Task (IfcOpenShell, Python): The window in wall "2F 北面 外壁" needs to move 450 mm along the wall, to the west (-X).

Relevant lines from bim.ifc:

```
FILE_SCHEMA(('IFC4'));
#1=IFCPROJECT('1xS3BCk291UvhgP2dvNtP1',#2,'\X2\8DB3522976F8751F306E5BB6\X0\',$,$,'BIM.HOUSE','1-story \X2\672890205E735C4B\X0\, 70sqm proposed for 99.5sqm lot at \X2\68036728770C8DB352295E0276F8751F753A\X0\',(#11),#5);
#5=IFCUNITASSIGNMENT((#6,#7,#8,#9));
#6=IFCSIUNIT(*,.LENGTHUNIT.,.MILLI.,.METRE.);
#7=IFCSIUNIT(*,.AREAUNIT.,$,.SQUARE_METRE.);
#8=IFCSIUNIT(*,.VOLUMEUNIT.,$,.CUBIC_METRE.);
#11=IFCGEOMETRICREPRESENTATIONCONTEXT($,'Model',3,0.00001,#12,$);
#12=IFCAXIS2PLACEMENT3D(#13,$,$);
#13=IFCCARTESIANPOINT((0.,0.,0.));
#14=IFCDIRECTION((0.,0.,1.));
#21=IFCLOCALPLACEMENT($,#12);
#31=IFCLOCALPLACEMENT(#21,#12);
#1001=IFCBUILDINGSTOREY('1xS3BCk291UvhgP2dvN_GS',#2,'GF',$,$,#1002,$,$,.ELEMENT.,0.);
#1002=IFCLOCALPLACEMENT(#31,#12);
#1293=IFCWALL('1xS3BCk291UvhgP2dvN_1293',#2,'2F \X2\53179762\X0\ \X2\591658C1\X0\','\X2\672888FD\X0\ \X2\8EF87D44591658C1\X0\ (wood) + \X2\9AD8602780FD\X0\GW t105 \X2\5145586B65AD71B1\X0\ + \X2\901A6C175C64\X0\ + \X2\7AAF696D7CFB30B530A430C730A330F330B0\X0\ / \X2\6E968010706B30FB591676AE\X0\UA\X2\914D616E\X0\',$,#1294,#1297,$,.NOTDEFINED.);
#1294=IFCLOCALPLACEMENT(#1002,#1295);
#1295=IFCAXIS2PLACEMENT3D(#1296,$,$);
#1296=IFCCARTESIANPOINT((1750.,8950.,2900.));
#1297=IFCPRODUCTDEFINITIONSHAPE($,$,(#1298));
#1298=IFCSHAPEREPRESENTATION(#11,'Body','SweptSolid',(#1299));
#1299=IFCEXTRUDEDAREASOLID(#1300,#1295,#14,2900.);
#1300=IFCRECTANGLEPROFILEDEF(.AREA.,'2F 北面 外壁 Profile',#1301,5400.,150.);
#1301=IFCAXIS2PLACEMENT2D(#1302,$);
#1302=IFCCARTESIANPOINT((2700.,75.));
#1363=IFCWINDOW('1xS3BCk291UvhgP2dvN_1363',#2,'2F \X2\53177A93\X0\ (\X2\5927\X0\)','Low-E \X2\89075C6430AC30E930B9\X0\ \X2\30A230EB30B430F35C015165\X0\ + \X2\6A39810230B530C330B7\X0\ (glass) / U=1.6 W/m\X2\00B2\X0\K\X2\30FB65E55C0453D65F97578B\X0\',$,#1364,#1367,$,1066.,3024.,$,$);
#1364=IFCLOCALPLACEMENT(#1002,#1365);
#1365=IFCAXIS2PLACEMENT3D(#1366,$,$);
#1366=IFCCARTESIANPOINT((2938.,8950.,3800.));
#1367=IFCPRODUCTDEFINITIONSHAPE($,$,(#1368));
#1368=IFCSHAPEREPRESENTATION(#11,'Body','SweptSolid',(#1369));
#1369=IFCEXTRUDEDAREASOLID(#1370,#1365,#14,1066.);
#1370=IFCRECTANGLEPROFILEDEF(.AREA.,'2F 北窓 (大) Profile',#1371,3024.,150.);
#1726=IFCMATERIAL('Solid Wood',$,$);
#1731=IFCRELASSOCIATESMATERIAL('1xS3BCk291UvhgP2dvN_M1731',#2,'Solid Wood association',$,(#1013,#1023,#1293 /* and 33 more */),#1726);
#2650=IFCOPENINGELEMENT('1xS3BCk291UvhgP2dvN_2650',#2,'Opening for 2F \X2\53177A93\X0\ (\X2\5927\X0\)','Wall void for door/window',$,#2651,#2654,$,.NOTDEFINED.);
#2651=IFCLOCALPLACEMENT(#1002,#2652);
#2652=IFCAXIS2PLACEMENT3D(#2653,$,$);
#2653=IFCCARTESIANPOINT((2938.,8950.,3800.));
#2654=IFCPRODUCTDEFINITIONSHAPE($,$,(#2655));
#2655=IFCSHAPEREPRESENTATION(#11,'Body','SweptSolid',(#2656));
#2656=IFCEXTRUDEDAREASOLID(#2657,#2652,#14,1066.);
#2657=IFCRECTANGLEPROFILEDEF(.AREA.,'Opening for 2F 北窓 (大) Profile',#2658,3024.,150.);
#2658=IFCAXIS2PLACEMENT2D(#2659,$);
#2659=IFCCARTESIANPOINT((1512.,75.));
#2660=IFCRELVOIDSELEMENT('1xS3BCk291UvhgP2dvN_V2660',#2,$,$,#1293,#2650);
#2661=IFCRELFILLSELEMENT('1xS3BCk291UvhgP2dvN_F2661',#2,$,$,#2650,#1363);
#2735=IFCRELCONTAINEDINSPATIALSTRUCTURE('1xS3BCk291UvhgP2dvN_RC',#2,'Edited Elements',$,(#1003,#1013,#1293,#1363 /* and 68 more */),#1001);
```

```python
import ifcopenshell
import ifcopenshell.api.geometry
import ifcopenshell.util.placement
import ifcopenshell.util.unit

model = ifcopenshell.open("bim.ifc")
unit_scale = ifcopenshell.util.unit.calculate_unit_scale(model)

window = model.by_guid("1xS3BCk291UvhgP2dvN_1363")
opening = window.FillsVoids[0].RelatingOpeningElement
wall = opening.VoidsElements[0].RelatingBuildingElement

wall_matrix = ifcopenshell.util.placement.get_local_placement(wall.ObjectPlacement)
shift = wall_matrix[:3, 0] * -0.45 / unit_scale
before = ifcopenshell.util.placement.get_local_placement(window.ObjectPlacement)[:3, 3].copy()

# The window is not placed relative to its opening, so move both.
for product in (opening, window):
    matrix = ifcopenshell.util.placement.get_local_placement(product.ObjectPlacement)
    matrix[:3, 3] += shift
    ifcopenshell.api.geometry.edit_object_placement(model, product=product, matrix=matrix, is_si=False)

after = ifcopenshell.util.placement.get_local_placement(window.ObjectPlacement)[:3, 3]
print("window moved by", (after - before).round(3) + 0.0)

model.write("bim_rev.ifc")
```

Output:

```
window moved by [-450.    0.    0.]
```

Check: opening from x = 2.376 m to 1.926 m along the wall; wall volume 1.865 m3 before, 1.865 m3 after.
